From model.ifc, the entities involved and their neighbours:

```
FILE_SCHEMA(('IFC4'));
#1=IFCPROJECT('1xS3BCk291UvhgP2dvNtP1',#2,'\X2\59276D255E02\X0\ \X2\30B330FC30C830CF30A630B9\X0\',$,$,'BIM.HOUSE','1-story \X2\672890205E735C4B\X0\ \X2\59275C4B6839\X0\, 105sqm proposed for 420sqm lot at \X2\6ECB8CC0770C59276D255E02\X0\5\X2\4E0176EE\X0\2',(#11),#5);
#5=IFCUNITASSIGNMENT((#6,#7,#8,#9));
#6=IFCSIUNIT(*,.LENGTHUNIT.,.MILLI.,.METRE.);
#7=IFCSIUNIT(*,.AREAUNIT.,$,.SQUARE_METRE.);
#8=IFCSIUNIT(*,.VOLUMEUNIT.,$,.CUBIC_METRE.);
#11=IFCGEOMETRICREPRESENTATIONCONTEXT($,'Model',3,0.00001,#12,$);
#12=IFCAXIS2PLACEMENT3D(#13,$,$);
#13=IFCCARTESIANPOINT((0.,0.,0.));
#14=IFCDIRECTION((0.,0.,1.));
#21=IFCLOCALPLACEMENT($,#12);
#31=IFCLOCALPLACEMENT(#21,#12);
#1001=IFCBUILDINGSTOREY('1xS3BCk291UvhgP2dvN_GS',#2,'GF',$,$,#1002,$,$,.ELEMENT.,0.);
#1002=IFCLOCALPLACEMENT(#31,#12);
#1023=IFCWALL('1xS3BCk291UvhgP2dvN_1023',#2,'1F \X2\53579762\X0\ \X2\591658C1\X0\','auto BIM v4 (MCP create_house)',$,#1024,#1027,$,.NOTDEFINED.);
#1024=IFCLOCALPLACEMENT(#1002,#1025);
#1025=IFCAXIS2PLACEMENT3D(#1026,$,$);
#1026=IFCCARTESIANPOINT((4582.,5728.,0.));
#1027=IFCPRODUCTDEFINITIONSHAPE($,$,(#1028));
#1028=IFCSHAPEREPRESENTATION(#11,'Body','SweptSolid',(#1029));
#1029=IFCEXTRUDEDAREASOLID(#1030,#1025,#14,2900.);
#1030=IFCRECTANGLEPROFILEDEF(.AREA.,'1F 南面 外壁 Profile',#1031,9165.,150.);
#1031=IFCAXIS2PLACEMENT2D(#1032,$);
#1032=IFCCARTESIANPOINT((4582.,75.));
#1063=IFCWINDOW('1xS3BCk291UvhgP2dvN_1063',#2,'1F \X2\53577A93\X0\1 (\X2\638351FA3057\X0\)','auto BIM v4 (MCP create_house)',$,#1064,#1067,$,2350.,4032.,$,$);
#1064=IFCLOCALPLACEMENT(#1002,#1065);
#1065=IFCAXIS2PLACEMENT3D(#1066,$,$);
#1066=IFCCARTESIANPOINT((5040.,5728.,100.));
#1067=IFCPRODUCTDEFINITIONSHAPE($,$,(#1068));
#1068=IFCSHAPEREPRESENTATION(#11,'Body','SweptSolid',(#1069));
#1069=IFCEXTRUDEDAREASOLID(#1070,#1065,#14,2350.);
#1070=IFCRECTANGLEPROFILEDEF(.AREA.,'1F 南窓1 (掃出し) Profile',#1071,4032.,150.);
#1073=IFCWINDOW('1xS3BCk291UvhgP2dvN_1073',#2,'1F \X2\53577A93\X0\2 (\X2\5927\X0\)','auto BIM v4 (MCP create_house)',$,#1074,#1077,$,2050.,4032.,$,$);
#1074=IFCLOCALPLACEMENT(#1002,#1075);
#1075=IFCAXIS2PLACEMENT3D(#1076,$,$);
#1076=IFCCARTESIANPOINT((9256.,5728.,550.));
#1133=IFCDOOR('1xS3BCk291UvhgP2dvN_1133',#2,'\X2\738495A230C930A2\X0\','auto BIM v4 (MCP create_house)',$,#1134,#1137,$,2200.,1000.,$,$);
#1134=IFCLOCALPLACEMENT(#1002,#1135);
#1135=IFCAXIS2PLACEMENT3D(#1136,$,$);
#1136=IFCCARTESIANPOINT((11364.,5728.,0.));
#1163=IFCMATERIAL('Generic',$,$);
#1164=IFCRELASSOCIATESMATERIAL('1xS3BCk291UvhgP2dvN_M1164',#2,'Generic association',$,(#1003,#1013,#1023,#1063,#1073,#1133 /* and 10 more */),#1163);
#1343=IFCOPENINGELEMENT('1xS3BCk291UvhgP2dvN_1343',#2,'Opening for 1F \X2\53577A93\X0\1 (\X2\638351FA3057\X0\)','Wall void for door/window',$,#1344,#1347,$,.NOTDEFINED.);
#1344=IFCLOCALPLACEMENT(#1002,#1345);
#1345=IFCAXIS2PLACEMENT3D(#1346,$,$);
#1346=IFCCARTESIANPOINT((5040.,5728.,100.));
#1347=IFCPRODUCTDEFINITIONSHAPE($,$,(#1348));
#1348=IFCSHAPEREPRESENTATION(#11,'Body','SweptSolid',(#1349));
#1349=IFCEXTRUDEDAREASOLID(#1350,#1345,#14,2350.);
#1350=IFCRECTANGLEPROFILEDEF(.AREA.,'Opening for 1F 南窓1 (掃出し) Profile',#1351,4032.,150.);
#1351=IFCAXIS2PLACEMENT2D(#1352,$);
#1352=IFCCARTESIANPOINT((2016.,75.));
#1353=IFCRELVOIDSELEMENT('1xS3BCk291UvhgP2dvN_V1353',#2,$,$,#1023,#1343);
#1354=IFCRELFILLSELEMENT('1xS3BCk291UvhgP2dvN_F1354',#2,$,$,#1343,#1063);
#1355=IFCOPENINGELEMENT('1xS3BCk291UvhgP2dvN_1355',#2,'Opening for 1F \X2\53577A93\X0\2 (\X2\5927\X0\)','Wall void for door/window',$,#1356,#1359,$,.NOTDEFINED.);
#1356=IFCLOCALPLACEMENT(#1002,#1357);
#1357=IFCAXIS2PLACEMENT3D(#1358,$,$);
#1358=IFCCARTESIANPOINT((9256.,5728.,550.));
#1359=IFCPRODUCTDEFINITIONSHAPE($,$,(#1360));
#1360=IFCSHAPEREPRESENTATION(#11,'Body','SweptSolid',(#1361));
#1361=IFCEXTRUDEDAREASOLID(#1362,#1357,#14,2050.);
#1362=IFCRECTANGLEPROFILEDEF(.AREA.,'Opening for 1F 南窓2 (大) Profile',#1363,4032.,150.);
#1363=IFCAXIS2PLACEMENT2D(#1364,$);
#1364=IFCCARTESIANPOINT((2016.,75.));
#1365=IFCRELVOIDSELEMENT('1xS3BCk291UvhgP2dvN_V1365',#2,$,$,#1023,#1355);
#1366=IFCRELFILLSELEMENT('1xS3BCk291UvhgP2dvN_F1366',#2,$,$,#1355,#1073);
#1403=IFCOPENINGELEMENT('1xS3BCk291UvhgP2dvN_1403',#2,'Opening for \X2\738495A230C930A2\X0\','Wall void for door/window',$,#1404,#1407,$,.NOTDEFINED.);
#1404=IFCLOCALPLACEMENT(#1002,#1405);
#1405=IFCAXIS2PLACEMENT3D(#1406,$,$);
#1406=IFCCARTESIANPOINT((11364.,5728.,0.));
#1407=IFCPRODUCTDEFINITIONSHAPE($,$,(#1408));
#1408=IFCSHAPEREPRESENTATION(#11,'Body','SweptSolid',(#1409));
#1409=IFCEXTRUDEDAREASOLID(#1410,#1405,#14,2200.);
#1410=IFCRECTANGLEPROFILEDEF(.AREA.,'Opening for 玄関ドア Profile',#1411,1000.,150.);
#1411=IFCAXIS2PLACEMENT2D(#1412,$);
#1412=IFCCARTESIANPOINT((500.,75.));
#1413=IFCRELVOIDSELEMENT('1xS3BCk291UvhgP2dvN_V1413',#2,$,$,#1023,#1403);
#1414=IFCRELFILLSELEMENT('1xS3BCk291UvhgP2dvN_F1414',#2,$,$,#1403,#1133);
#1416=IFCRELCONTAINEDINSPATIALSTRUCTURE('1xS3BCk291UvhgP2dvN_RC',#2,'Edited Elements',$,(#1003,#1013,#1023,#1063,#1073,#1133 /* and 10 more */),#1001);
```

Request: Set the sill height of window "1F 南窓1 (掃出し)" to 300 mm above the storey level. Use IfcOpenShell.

```python
import numpy as np
import ifcopenshell
import ifcopenshell.api.geometry
import ifcopenshell.geom
import ifcopenshell.util.element
import ifcopenshell.util.placement
import ifcopenshell.util.shape
import ifcopenshell.util.unit

model = ifcopenshell.open("model.ifc")
unit_scale = ifcopenshell.util.unit.calculate_unit_scale(model)

window = model.by_guid("1xS3BCk291UvhgP2dvN_1063")
opening = window.FillsVoids[0].RelatingOpeningElement
storey = ifcopenshell.util.element.get_container(window, ifc_class="IfcBuildingStorey")
level = ifcopenshell.util.placement.get_local_placement(storey.ObjectPlacement)[2, 3]

# The opening's origin need not be at the sill, so measure its lowest point.
shape = ifcopenshell.geom.create_shape(ifcopenshell.geom.settings(), opening)
bottom = ifcopenshell.util.shape.get_shape_bottom_elevation(shape, shape.geometry) / unit_scale
dz = level + 0.3 / unit_scale - bottom

shift = np.array([0.0, 0.0, dz])
# The window is not placed relative to its opening, so move both.
for product in (opening, window):
    matrix = ifcopenshell.util.placement.get_local_placement(product.ObjectPlacement)
    matrix[:3, 3] += shift
    ifcopenshell.api.geometry.edit_object_placement(model, product=product, matrix=matrix, is_si=False)

print(f"moved by {dz * unit_scale:+.3f} m")

model.write("model-out.ifc")
```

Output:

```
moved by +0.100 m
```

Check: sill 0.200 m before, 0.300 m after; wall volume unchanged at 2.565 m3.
